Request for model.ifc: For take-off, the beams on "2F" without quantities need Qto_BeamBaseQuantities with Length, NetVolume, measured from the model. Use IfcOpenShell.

First a look at what the model holds.

```python
import ifcopenshell
import ifcopenshell.util.element
import ifcopenshell.util.unit

model = ifcopenshell.open("model.ifc")
print(model.schema)
for unit_type in ("LENGTHUNIT", "AREAUNIT", "VOLUMEUNIT"):
    print(unit_type, ifcopenshell.util.unit.calculate_unit_scale(model, unit_type))
storey = next(s for s in model.by_type("IfcBuildingStorey") if s.Name == "2F")
beams = [e for e in ifcopenshell.util.element.get_decomposition(storey) if e.is_a("IfcBeam")]
for e in sorted(beams, key=lambda e: e.id()):
    print(e.id(), e.is_a(), e.Name, list(ifcopenshell.util.element.get_psets(e, qtos_only=True)), sep=" | ")
```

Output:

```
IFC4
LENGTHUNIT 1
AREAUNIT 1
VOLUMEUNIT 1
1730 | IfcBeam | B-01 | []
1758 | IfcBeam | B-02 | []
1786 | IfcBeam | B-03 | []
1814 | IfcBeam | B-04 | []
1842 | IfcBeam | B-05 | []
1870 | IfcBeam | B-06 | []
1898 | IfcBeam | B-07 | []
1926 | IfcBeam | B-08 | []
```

```python
import ifcopenshell
import ifcopenshell.api.pset
import ifcopenshell.geom
import ifcopenshell.util.element
import ifcopenshell.util.shape
import ifcopenshell.util.unit

model = ifcopenshell.open("model.ifc")
unit_scale = ifcopenshell.util.unit.calculate_unit_scale(model)
volume_scale = ifcopenshell.util.unit.calculate_unit_scale(model, "VOLUMEUNIT")
settings = ifcopenshell.geom.settings()

storey = next(s for s in model.by_type("IfcBuildingStorey") if s.Name == "2F")
beams = [e for e in ifcopenshell.util.element.get_decomposition(storey) if e.is_a("IfcBeam")]

for e in sorted(beams, key=lambda e: e.id()):
    if ifcopenshell.util.element.get_psets(e, qtos_only=True, should_inherit=False):
        continue
    # Geometry comes back in metres, in the element's own axes.
    shape = ifcopenshell.geom.create_shape(settings, e)
    values = {
        "Length": ifcopenshell.util.shape.get_max_xyz(shape.geometry) / unit_scale,
        "NetVolume": ifcopenshell.util.shape.get_volume(shape.geometry) / volume_scale,
    }
    qto = ifcopenshell.api.pset.add_qto(model, product=e, name="Qto_BeamBaseQuantities")
    ifcopenshell.api.pset.edit_qto(model, qto=qto, properties=values)
    print(e.id(), {k: round(v, 3) for k, v in values.items()})

model.write("model-out.ifc")
```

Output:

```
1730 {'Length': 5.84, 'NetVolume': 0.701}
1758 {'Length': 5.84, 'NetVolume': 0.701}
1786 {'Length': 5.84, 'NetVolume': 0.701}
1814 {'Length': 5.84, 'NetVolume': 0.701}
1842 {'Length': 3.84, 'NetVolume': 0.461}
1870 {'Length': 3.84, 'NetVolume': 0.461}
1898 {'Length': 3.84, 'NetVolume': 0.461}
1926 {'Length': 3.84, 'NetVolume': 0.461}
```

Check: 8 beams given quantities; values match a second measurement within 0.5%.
